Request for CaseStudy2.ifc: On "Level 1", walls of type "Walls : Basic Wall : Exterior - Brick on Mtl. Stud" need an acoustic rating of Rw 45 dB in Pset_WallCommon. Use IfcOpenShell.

First a look at what the model holds.

```python
import ifcopenshell
import ifcopenshell.util.element

model = ifcopenshell.open("CaseStudy2.ifc")
print(model.schema)
storey = next(s for s in model.by_type("IfcBuildingStorey") if s.Name == "Level 1")
walls = [e for e in ifcopenshell.util.element.get_decomposition(storey) if e.is_a("IfcWall")]
seen = {}
for e in walls:
    element_type = ifcopenshell.util.element.get_type(e)
    key = (element_type.Name if element_type != e and element_type else None, ifcopenshell.util.element.get_pset(e, "Pset_WallCommon", "AcousticRating"))
    seen[key] = seen.get(key, 0) + 1
for (name, value), count in sorted(seen.items(), key=str):
    print(count, "x", name, "|", value)
```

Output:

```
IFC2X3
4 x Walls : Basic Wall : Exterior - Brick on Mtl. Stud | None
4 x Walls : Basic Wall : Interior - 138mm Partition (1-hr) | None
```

```python
import ifcopenshell
import ifcopenshell.api.pset
import ifcopenshell.util.element

model = ifcopenshell.open("CaseStudy2.ifc")

storey = next(s for s in model.by_type("IfcBuildingStorey") if s.Name == "Level 1")
walls = [e for e in ifcopenshell.util.element.get_decomposition(storey) if e.is_a("IfcWall")]

count = 0
for e in walls:
    element_type = ifcopenshell.util.element.get_type(e)
    if element_type in (None, e) or element_type.Name != "Walls : Basic Wall : Exterior - Brick on Mtl. Stud":
        continue
    # add_pset returns the element's existing set when there is one.
    pset = ifcopenshell.api.pset.add_pset(model, product=e, name="Pset_WallCommon")
    ifcopenshell.api.pset.edit_pset(model, pset=pset, properties={"AcousticRating": "Rw 45 dB"})
    count += 1

print(count, "walls updated")

model.write("CaseStudy2_edited.ifc")
```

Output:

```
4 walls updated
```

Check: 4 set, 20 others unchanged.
